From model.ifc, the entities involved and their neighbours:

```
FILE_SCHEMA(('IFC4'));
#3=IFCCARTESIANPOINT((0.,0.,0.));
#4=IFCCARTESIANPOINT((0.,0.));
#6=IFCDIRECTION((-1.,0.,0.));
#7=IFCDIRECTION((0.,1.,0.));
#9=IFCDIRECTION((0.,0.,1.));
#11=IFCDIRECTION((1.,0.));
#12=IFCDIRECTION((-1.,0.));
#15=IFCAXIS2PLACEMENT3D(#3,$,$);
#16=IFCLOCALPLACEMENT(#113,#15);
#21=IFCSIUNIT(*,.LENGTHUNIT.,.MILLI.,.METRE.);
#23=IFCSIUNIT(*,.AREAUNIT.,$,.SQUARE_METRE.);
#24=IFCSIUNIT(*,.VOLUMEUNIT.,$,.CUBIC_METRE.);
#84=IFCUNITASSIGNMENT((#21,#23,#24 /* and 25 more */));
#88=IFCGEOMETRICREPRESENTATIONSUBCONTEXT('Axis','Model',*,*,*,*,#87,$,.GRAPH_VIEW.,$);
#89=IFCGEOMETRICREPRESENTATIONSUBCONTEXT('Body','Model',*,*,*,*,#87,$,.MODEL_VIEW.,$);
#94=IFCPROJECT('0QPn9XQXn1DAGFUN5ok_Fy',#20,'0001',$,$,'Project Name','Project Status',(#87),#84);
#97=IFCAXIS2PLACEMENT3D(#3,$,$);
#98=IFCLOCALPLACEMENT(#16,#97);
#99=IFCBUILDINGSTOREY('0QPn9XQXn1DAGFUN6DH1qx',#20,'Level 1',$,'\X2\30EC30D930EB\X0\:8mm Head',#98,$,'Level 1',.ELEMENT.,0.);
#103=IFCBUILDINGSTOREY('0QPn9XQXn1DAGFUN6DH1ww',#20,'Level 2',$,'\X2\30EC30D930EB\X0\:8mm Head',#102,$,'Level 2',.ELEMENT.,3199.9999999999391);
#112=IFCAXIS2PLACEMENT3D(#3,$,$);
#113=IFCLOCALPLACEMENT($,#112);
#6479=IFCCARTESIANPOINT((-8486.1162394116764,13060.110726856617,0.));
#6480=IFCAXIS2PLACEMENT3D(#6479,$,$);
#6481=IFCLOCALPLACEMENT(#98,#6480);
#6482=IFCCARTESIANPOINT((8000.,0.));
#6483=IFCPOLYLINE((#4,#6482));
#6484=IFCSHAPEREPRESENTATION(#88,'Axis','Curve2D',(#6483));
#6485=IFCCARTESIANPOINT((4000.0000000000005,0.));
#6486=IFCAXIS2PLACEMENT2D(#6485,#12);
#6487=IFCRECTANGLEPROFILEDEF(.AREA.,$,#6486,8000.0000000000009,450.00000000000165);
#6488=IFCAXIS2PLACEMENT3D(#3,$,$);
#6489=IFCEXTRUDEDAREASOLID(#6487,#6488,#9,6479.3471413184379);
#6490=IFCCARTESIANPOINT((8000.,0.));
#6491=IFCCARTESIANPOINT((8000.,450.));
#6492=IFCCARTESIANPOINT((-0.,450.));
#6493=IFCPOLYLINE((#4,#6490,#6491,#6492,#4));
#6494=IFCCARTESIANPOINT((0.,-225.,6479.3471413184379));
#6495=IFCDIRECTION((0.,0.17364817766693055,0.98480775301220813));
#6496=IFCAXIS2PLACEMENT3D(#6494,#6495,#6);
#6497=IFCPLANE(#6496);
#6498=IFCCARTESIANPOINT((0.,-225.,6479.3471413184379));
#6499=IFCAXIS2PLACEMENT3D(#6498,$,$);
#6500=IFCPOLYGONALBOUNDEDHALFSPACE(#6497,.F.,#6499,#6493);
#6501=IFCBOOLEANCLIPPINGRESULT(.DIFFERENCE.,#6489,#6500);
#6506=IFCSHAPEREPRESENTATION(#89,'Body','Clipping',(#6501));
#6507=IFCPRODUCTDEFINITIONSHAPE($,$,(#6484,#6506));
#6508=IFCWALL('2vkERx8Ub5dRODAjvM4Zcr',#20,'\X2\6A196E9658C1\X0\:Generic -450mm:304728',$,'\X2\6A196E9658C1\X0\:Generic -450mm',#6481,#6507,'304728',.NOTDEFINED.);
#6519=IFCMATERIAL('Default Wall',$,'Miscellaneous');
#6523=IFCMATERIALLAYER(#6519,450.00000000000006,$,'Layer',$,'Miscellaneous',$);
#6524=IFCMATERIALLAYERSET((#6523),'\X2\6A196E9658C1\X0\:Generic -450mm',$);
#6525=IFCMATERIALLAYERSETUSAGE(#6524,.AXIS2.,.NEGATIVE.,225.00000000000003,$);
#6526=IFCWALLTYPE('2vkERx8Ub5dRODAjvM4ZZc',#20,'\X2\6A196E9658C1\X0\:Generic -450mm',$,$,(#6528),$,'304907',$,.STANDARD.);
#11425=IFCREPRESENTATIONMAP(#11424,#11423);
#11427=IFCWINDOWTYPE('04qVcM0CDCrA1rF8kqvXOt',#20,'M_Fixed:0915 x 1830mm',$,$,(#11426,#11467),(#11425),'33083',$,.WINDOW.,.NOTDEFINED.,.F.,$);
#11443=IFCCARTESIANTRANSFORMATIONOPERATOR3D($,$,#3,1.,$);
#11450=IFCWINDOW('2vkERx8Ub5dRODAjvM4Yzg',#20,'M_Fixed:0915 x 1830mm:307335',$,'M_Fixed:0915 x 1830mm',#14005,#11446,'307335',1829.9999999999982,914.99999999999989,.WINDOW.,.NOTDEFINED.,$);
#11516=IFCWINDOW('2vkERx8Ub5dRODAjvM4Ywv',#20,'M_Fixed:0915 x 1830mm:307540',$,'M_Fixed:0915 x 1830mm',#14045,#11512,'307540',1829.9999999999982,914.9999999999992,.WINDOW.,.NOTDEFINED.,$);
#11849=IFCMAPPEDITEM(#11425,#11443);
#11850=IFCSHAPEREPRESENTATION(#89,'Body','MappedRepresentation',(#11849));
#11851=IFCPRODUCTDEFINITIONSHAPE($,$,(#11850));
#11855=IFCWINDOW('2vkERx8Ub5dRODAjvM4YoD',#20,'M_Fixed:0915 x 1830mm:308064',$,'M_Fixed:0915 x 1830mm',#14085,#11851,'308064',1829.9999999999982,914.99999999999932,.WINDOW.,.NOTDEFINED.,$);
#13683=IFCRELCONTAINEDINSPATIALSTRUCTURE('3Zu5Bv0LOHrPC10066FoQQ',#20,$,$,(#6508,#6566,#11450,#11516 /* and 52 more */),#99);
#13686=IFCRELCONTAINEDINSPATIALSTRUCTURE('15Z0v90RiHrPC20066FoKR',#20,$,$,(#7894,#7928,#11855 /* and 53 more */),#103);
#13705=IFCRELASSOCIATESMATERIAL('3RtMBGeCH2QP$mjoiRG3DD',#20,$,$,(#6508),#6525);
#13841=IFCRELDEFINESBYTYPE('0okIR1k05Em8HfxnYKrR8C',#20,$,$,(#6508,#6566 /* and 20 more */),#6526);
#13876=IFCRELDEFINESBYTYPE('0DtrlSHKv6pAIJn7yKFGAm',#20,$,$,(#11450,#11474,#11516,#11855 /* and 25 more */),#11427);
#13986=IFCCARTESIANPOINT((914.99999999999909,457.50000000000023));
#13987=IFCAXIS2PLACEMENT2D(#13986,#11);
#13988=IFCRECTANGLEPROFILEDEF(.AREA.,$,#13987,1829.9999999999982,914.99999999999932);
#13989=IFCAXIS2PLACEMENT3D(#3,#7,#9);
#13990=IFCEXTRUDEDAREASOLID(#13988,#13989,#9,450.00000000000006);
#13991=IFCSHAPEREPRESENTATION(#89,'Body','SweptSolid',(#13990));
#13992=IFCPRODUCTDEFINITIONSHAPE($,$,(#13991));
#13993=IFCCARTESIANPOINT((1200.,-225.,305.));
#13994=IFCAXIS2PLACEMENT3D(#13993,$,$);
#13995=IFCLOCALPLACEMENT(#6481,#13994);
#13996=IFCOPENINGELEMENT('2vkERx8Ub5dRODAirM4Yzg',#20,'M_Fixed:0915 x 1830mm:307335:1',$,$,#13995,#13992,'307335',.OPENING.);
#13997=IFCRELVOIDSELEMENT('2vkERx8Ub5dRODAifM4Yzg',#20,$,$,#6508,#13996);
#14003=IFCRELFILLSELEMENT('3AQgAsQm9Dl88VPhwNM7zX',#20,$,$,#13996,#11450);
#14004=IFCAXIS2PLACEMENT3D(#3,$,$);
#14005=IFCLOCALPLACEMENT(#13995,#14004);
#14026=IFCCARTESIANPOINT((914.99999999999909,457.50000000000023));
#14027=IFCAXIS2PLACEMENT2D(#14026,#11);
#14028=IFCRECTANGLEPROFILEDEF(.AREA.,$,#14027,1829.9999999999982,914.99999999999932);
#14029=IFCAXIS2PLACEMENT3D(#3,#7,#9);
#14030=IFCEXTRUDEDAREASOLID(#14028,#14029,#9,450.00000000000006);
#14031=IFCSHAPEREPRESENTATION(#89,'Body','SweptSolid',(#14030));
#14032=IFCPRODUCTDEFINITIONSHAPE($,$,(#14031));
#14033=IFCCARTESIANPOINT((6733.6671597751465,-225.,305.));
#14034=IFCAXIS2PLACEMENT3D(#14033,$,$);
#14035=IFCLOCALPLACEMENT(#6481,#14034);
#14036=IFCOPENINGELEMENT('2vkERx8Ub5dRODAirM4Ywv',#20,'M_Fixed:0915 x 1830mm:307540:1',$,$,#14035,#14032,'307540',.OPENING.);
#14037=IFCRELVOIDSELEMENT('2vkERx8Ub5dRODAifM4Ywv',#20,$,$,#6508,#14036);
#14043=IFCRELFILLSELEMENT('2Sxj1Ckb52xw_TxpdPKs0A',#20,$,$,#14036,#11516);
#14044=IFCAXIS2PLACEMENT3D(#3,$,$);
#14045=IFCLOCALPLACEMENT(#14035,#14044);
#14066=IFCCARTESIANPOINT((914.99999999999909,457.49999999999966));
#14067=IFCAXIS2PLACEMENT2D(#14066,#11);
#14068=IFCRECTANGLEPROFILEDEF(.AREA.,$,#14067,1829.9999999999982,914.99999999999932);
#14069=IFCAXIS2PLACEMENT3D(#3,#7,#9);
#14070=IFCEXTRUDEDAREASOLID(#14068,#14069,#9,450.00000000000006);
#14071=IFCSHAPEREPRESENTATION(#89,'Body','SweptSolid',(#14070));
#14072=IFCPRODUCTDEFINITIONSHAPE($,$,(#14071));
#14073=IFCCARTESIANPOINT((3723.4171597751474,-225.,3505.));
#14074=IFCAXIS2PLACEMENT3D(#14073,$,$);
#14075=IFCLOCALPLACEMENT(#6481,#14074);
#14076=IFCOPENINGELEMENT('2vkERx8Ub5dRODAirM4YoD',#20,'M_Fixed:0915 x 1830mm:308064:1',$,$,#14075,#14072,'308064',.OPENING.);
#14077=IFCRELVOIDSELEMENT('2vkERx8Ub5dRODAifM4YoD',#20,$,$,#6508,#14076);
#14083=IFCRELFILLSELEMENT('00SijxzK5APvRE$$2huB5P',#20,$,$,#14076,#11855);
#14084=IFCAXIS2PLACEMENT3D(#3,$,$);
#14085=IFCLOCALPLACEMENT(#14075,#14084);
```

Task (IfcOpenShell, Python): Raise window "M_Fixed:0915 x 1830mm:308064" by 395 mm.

```python
import numpy as np
import ifcopenshell
import ifcopenshell.api.geometry
import ifcopenshell.util.placement
import ifcopenshell.util.unit

model = ifcopenshell.open("model.ifc")
unit_scale = ifcopenshell.util.unit.calculate_unit_scale(model)

window = model.by_guid("2vkERx8Ub5dRODAjvM4YoD")
opening = window.FillsVoids[0].RelatingOpeningElement
dz = 395.0

shift = np.array([0.0, 0.0, dz])
# The window is placed relative to its opening, so it follows when the opening moves.
matrix = ifcopenshell.util.placement.get_local_placement(opening.ObjectPlacement)
matrix[:3, 3] += shift
ifcopenshell.api.geometry.edit_object_placement(
    model, product=opening, matrix=matrix, is_si=False, should_transform_children=True
)

print(f"moved by {dz * unit_scale:+.3f} m")

model.write("model-out.ifc")
```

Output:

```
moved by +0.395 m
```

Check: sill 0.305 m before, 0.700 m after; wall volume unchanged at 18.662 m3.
